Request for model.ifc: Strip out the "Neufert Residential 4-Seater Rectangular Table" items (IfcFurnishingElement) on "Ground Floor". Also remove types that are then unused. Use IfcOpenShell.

First a look at what the model holds.

```python
import ifcopenshell
import ifcopenshell.util.element

model = ifcopenshell.open("model.ifc")
print(model.schema)
storey = next(s for s in model.by_type("IfcBuildingStorey") if s.Name == "Ground Floor")
furniture = [e for e in ifcopenshell.util.element.get_decomposition(storey) if e.is_a("IfcFurnishingElement")]
seen = {}
for e in furniture:
    element_type = ifcopenshell.util.element.get_type(e)
    name = element_type.Name if element_type not in (None, e) else None
    seen[name] = seen.get(name, 0) + 1
for name, count in sorted(seen.items(), key=str):
    print(count, "x", name)
```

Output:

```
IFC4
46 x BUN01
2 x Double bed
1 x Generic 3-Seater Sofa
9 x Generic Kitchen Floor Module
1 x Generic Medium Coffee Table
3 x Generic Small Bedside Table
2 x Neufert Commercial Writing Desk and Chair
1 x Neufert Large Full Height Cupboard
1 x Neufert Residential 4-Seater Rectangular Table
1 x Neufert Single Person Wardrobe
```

```python
import ifcopenshell
import ifcopenshell.api.root
import ifcopenshell.util.element

model = ifcopenshell.open("model.ifc")

storey = next(s for s in model.by_type("IfcBuildingStorey") if s.Name == "Ground Floor")
furniture = [e for e in ifcopenshell.util.element.get_decomposition(storey) if e.is_a("IfcFurnishingElement")]
targets = [e for e in furniture if (t := ifcopenshell.util.element.get_type(e)) not in (None, e) and t.Name == "Neufert Residential 4-Seater Rectangular Table"]
types = {ifcopenshell.util.element.get_type(e) for e in targets} - {None, *targets}

for e in targets:
    ifcopenshell.api.root.remove_product(model, product=e)
print(len(targets), "removed")

unused = [t for t in types if not ifcopenshell.util.element.get_types(t)]
for t in unused:
    ifcopenshell.api.root.remove_product(model, product=t)
print(len(unused), "unused types removed")

model.write("model_v2.ifc")
```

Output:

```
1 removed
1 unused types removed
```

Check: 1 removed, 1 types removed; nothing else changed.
